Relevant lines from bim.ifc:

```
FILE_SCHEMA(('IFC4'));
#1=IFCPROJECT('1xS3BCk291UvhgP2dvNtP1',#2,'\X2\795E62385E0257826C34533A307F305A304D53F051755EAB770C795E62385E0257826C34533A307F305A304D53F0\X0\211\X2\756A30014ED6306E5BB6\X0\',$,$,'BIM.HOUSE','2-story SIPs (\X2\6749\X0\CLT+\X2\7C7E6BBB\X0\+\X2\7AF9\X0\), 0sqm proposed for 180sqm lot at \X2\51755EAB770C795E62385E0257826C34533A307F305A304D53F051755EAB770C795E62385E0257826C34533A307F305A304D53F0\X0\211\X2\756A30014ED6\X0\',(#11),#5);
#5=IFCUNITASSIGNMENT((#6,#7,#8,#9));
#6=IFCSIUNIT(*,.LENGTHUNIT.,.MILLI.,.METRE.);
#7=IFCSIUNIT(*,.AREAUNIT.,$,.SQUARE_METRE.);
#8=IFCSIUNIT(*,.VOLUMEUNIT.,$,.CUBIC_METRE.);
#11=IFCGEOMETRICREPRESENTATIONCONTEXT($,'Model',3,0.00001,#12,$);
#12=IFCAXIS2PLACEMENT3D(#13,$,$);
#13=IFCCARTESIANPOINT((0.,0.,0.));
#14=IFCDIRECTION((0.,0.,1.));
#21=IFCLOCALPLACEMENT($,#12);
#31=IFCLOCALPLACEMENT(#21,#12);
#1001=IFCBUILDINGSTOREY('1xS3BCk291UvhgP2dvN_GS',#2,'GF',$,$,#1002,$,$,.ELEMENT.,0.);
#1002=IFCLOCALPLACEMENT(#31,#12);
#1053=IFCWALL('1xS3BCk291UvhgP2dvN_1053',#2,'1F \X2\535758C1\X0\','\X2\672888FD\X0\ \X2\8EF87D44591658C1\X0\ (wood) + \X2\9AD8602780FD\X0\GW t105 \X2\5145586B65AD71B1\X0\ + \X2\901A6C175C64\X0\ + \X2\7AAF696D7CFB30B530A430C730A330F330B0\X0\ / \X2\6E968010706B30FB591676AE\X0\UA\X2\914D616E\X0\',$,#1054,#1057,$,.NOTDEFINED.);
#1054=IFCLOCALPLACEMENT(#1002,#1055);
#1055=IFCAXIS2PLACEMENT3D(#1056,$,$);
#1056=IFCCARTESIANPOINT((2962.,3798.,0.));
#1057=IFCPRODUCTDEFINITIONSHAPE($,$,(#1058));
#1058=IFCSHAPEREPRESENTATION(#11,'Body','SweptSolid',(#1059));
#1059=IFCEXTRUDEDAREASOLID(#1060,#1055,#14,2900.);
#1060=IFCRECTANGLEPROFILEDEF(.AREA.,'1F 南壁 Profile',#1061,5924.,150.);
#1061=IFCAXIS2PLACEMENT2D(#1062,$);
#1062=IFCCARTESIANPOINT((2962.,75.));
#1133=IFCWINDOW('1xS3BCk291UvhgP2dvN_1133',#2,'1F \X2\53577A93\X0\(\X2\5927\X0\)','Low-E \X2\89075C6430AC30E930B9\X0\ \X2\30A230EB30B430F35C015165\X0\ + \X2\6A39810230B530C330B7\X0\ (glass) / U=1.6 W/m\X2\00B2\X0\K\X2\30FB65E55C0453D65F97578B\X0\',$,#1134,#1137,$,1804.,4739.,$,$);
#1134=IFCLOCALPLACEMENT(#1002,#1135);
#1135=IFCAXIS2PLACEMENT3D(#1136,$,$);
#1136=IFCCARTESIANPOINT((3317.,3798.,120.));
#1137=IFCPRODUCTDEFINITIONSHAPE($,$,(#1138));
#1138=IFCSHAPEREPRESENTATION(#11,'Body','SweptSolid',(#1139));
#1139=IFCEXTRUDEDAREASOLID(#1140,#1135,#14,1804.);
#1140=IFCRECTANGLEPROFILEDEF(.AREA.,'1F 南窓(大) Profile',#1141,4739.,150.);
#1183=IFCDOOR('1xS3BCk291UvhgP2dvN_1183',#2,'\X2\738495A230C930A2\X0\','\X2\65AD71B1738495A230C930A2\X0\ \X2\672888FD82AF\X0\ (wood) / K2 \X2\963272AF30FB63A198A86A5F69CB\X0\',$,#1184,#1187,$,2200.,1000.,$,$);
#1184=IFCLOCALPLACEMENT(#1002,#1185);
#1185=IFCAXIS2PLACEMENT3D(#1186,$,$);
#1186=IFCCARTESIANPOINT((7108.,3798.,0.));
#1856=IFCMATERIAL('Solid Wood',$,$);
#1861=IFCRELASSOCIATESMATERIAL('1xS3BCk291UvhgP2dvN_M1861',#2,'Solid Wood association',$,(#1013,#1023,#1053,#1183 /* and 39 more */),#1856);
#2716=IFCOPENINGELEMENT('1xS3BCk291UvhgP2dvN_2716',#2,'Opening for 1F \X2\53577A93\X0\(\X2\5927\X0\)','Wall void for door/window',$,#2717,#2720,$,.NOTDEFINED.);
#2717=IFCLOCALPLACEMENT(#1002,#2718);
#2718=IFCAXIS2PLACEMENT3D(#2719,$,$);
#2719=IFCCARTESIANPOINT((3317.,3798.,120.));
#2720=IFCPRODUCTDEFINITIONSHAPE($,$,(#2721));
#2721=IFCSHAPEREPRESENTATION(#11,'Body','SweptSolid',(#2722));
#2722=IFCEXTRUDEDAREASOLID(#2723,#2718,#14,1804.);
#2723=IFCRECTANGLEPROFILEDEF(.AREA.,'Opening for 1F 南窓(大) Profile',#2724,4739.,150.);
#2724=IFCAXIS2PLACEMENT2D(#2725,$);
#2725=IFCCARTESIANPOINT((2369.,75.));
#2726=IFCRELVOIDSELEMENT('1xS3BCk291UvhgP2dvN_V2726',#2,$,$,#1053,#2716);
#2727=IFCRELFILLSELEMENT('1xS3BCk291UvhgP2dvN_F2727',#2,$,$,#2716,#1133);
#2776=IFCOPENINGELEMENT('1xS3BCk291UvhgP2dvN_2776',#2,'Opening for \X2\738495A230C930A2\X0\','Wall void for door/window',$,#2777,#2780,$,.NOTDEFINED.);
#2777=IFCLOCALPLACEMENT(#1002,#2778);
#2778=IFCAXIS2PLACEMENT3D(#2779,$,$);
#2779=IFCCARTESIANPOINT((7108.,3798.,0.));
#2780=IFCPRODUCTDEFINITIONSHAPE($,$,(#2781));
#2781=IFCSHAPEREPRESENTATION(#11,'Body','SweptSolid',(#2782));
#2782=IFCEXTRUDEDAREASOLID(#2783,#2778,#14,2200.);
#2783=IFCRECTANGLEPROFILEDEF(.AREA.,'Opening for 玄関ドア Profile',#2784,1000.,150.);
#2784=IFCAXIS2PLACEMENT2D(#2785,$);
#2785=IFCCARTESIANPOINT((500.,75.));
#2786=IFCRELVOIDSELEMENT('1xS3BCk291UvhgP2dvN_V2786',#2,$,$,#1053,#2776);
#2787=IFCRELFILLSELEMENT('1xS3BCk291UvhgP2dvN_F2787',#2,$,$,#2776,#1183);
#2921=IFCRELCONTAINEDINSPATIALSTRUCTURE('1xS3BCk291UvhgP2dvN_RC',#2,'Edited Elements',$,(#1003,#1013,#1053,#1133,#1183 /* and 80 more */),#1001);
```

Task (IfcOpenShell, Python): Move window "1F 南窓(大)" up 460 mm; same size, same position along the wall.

```python
import numpy as np
import ifcopenshell
import ifcopenshell.api.geometry
import ifcopenshell.util.placement
import ifcopenshell.util.unit

model = ifcopenshell.open("bim.ifc")
unit_scale = ifcopenshell.util.unit.calculate_unit_scale(model)

window = model.by_guid("1xS3BCk291UvhgP2dvN_1133")
opening = window.FillsVoids[0].RelatingOpeningElement
dz = 460.0

shift = np.array([0.0, 0.0, dz])
# The window is not placed relative to its opening, so move both.
for product in (opening, window):
    matrix = ifcopenshell.util.placement.get_local_placement(product.ObjectPlacement)
    matrix[:3, 3] += shift
    ifcopenshell.api.geometry.edit_object_placement(model, product=product, matrix=matrix, is_si=False)

print(f"moved by {dz * unit_scale:+.3f} m")

model.write("bim_rev.ifc")
```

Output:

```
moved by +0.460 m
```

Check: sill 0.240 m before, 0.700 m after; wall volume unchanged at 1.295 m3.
